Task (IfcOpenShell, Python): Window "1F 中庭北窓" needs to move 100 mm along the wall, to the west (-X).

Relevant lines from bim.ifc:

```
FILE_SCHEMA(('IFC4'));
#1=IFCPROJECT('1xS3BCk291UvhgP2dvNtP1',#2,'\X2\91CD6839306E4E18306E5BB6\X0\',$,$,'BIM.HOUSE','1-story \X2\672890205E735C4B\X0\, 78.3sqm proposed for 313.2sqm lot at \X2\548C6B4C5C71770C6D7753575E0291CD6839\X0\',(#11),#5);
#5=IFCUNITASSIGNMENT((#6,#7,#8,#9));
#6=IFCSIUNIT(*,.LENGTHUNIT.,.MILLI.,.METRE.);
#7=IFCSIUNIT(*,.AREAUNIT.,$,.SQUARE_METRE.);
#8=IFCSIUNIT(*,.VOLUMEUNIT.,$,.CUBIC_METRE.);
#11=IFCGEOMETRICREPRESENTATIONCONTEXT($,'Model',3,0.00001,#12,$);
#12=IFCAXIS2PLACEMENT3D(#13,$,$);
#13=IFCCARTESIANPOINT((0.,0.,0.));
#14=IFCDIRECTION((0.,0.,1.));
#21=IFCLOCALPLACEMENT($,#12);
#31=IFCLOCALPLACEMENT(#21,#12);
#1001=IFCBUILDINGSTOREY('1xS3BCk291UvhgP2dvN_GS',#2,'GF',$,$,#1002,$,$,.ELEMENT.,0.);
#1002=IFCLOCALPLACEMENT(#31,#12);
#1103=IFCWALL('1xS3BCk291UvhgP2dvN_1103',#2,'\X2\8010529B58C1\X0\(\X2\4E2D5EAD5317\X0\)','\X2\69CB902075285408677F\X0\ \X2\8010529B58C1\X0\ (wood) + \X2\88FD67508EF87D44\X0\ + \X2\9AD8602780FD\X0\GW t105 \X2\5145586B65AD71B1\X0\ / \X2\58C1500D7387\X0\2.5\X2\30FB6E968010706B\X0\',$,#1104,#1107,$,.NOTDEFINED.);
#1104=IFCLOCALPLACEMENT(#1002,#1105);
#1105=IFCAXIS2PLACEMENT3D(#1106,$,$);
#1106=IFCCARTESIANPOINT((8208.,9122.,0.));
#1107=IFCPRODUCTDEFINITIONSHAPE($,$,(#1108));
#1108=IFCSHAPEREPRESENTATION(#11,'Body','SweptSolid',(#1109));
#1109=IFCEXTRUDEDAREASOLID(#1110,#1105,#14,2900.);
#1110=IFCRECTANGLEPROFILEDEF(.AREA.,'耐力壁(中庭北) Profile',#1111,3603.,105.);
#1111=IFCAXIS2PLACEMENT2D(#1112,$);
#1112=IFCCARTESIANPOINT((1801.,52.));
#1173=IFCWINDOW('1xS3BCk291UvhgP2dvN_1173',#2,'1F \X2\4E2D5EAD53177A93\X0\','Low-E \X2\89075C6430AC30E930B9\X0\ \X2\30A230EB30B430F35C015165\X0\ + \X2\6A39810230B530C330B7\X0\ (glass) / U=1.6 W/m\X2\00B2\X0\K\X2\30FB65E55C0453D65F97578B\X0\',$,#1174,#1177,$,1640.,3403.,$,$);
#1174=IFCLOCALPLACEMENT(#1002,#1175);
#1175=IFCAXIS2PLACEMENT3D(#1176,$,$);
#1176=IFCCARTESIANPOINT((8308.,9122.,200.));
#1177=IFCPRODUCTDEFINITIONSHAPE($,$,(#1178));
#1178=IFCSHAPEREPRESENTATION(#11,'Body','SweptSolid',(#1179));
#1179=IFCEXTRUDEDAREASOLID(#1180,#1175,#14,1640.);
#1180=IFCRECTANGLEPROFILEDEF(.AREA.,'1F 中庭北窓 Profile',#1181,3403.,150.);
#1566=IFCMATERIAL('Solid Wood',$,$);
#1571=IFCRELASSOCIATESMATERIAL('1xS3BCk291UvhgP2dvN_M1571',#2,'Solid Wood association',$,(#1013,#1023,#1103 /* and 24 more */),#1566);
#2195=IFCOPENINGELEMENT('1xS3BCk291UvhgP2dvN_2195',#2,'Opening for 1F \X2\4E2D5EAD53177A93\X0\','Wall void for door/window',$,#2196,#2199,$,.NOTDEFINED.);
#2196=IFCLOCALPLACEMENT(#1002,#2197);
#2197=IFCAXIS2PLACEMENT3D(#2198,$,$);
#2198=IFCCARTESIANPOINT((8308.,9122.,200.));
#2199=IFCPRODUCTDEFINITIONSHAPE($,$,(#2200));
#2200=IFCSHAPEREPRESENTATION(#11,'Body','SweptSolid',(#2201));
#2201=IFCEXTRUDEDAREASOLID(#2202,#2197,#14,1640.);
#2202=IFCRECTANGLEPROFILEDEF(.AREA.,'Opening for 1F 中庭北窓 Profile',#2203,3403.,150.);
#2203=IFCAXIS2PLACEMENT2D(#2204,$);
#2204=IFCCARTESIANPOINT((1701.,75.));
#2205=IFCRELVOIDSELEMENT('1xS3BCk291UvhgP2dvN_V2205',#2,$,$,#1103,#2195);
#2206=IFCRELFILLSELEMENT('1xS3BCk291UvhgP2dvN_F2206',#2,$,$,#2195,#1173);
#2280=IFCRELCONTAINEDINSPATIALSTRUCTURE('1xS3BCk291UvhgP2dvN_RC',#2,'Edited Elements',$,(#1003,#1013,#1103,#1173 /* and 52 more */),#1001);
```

```python
import ifcopenshell
import ifcopenshell.api.geometry
import ifcopenshell.util.placement
import ifcopenshell.util.unit

model = ifcopenshell.open("bim.ifc")
unit_scale = ifcopenshell.util.unit.calculate_unit_scale(model)

window = model.by_guid("1xS3BCk291UvhgP2dvN_1173")
opening = window.FillsVoids[0].RelatingOpeningElement
wall = opening.VoidsElements[0].RelatingBuildingElement

wall_matrix = ifcopenshell.util.placement.get_local_placement(wall.ObjectPlacement)
shift = wall_matrix[:3, 0] * -0.1 / unit_scale
before = ifcopenshell.util.placement.get_local_placement(window.ObjectPlacement)[:3, 3].copy()

# The window is not placed relative to its opening, so move both.
for product in (opening, window):
    matrix = ifcopenshell.util.placement.get_local_placement(product.ObjectPlacement)
    matrix[:3, 3] += shift
    ifcopenshell.api.geometry.edit_object_placement(model, product=product, matrix=matrix, is_si=False)

after = ifcopenshell.util.placement.get_local_placement(window.ObjectPlacement)[:3, 3]
print("window moved by", (after - before).round(3) + 0.0)

model.write("bim_rev.ifc")
```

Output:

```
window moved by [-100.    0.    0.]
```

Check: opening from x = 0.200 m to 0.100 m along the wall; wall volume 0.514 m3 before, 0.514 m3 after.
